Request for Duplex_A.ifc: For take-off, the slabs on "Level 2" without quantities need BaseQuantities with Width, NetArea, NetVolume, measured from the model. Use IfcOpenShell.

First a look at what the model holds.

```python
import ifcopenshell
import ifcopenshell.util.element
import ifcopenshell.util.unit

model = ifcopenshell.open("Duplex_A.ifc")
print(model.schema)
for unit_type in ("LENGTHUNIT", "AREAUNIT", "VOLUMEUNIT"):
    print(unit_type, ifcopenshell.util.unit.calculate_unit_scale(model, unit_type))
storey = next(s for s in model.by_type("IfcBuildingStorey") if s.Name == "Level 2")
slabs = [e for e in ifcopenshell.util.element.get_decomposition(storey) if e.is_a("IfcSlab")]
for e in sorted(slabs, key=lambda e: e.id()):
    print(e.id(), e.is_a(), e.Name, list(ifcopenshell.util.element.get_psets(e, qtos_only=True)), sep=" | ")
```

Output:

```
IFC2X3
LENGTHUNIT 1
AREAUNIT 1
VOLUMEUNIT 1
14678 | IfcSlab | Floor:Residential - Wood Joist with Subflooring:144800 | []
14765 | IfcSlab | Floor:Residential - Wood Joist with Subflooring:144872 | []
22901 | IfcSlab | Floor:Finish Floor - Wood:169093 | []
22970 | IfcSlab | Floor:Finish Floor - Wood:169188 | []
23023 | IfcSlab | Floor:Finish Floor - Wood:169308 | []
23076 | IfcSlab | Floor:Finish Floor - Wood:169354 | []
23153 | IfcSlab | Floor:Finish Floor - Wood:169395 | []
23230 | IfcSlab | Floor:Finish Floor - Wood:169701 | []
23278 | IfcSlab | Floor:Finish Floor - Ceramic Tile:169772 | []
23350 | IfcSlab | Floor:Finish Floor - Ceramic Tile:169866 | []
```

```python
import ifcopenshell
import ifcopenshell.api.pset
import ifcopenshell.geom
import ifcopenshell.util.element
import ifcopenshell.util.shape
import ifcopenshell.util.unit

model = ifcopenshell.open("Duplex_A.ifc")
unit_scale = ifcopenshell.util.unit.calculate_unit_scale(model)
area_scale = ifcopenshell.util.unit.calculate_unit_scale(model, "AREAUNIT")
volume_scale = ifcopenshell.util.unit.calculate_unit_scale(model, "VOLUMEUNIT")
settings = ifcopenshell.geom.settings()

storey = next(s for s in model.by_type("IfcBuildingStorey") if s.Name == "Level 2")
slabs = [e for e in ifcopenshell.util.element.get_decomposition(storey) if e.is_a("IfcSlab")]

for e in sorted(slabs, key=lambda e: e.id()):
    if ifcopenshell.util.element.get_psets(e, qtos_only=True, should_inherit=False):
        continue
    # Geometry comes back in metres, in the element's own axes.
    shape = ifcopenshell.geom.create_shape(settings, e)
    values = {
        "Width": ifcopenshell.util.shape.get_z(shape.geometry) / unit_scale,
        "NetArea": ifcopenshell.util.shape.get_footprint_area(shape.geometry) / area_scale,
        "NetVolume": ifcopenshell.util.shape.get_volume(shape.geometry) / volume_scale,
    }
    qto = ifcopenshell.api.pset.add_qto(model, product=e, name="BaseQuantities")
    ifcopenshell.api.pset.edit_qto(model, qto=qto, properties=values)
    print(e.id(), {k: round(v, 3) for k, v in values.items()})

model.write("Duplex_A_v2.ifc")
```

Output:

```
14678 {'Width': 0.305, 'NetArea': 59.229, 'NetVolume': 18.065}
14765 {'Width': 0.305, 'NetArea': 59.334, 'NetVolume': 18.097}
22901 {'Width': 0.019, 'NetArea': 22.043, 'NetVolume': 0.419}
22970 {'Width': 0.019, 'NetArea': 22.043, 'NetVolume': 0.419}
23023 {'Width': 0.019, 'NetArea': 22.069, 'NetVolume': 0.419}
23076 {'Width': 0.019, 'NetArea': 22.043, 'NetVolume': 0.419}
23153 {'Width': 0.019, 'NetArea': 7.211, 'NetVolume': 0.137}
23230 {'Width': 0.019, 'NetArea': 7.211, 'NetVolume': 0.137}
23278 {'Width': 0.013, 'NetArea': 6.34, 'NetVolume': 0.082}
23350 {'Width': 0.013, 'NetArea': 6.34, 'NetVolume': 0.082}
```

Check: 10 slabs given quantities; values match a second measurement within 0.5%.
